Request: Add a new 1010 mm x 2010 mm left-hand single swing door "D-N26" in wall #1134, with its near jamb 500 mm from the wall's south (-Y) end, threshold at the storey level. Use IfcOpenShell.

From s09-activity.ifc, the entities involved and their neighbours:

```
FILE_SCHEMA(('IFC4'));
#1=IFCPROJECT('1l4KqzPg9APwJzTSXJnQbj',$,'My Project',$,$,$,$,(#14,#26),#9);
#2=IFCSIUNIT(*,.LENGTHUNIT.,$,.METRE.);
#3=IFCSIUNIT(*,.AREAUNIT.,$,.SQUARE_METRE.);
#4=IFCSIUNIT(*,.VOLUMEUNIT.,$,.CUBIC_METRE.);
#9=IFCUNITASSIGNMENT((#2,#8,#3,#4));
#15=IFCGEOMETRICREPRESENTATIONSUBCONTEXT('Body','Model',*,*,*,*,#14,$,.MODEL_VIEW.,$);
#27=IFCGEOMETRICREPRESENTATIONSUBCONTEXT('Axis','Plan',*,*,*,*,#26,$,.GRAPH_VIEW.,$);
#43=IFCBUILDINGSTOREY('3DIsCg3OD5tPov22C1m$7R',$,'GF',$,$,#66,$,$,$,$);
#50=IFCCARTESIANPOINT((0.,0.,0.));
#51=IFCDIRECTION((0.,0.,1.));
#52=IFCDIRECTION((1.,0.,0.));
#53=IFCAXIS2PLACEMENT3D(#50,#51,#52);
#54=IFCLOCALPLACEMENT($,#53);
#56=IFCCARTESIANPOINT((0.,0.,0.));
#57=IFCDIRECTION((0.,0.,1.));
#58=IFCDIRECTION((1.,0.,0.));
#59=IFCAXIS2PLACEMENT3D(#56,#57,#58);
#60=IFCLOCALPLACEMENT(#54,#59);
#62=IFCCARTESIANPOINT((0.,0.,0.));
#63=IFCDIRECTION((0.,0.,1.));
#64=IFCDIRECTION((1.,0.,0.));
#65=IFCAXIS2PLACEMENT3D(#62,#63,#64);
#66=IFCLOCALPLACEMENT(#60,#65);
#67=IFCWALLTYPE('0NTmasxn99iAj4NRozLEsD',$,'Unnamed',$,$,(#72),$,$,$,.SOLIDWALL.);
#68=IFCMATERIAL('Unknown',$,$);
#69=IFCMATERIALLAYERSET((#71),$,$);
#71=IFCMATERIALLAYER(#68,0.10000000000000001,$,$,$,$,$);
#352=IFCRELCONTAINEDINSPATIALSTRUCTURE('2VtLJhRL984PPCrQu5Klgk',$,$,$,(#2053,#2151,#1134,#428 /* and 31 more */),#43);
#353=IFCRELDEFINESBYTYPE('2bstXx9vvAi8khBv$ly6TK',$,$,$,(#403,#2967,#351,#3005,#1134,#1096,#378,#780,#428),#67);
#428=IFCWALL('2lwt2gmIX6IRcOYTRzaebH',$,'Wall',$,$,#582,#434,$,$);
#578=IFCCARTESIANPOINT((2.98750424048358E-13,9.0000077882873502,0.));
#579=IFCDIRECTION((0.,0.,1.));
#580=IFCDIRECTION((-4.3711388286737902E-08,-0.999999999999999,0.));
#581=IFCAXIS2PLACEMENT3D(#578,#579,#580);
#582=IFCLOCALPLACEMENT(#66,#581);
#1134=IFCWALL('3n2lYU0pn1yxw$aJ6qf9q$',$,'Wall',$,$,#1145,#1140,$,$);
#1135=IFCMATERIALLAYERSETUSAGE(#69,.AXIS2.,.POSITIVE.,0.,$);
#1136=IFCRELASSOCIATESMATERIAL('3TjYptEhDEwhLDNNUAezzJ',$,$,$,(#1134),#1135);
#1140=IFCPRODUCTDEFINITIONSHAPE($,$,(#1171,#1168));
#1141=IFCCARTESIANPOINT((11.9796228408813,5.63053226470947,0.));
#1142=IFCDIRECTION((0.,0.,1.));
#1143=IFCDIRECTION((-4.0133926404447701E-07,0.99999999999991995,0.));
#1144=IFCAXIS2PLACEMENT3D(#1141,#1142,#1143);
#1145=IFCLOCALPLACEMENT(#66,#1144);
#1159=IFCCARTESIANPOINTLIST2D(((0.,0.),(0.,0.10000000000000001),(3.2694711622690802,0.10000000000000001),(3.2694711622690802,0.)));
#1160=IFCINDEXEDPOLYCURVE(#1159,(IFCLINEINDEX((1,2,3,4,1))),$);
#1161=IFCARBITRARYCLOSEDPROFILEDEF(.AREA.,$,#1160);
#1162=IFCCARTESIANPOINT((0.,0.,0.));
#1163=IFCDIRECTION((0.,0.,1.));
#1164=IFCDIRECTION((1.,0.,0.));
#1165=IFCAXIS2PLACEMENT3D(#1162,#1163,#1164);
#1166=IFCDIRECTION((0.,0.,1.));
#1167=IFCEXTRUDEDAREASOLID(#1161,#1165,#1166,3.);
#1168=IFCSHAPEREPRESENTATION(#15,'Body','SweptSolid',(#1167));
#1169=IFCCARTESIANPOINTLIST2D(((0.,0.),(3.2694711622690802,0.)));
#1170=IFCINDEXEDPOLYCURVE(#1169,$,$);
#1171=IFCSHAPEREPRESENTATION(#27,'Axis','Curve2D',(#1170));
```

```python
import numpy as np
import ifcopenshell
import ifcopenshell.api.feature
import ifcopenshell.api.geometry
import ifcopenshell.api.root
import ifcopenshell.api.spatial
import ifcopenshell.geom
import ifcopenshell.util.element
import ifcopenshell.util.placement
import ifcopenshell.util.representation
import ifcopenshell.util.shape
import ifcopenshell.util.unit

model = ifcopenshell.open("s09-activity.ifc")
unit_scale = ifcopenshell.util.unit.calculate_unit_scale(model)
settings = ifcopenshell.geom.settings()


def volume(element):
    """Net volume in cubic metres, openings subtracted."""
    shape = ifcopenshell.geom.create_shape(settings, element)
    return ifcopenshell.util.shape.get_volume(shape.geometry)


wall = model.by_id(1134)
storey = ifcopenshell.util.element.get_container(wall, ifc_class="IfcBuildingStorey")
context = ifcopenshell.util.representation.get_context(model, "Model", "Body", "MODEL_VIEW")
before = volume(wall)

width, height, from_end, sill = 1.01, 2.01, 0.5, 0.0  # metres

# The wall runs along its own X axis, and the end named is its -X end.
wall_shape = ifcopenshell.geom.create_shape(settings, wall)
x, y, z = ifcopenshell.util.shape.get_vertices(wall_shape.geometry).T
start = x.min() + from_end
face, thickness = float(y.min()), float(y.max() - y.min())
wall_matrix = ifcopenshell.util.placement.get_local_placement(wall.ObjectPlacement)
level = ifcopenshell.util.placement.get_local_placement(storey.ObjectPlacement)[2, 3]


def in_wall(x, y):
    """Placement at x, y metres in the wall's axes, at sill height."""
    matrix = wall_matrix.copy()
    matrix[:, 3] = wall_matrix @ np.array([x / unit_scale, y / unit_scale, 0.0, 1.0])
    matrix[2, 3] = level + sill / unit_scale
    return matrix


# Opening: a box that overshoots both wall faces by 50 mm.
opening = ifcopenshell.api.root.create_entity(model, ifc_class="IfcOpeningElement", predefined_type="OPENING")
box = ifcopenshell.api.geometry.add_wall_representation(
    model, context=context, length=width, height=height, thickness=thickness + 0.1
)
ifcopenshell.api.geometry.assign_representation(model, product=opening, representation=box)
ifcopenshell.api.geometry.edit_object_placement(model, product=opening, matrix=in_wall(start, face - 0.05), is_si=False)
ifcopenshell.api.feature.add_feature(model, feature=opening, element=wall)

door = ifcopenshell.api.root.create_entity(model, ifc_class="IfcDoor", name="D-N26", predefined_type="DOOR")
door.OverallWidth, door.OverallHeight = width / unit_scale, height / unit_scale
door.OperationType = "SINGLE_SWING_LEFT"
body = ifcopenshell.api.geometry.add_door_representation(
    model,
    context=context,
    overall_width=door.OverallWidth,
    overall_height=door.OverallHeight,
    operation_type="SINGLE_SWING_LEFT",
    lining_properties={"LiningDepth": thickness / unit_scale, "ThresholdDepth": thickness / unit_scale},
)
ifcopenshell.api.geometry.assign_representation(model, product=door, representation=body)
ifcopenshell.api.spatial.assign_container(model, products=[door], relating_structure=storey)
ifcopenshell.api.feature.add_filling(model, opening=opening, element=door)

# The lining spans the wall, so the door starts at the wall face.
ifcopenshell.api.geometry.edit_object_placement(model, product=door, matrix=in_wall(start, face), is_si=False)

after = volume(wall)

print(f"wall volume {before:.3f} -> {after:.3f} m3")

model.write("s09-activity_v2.ifc")
```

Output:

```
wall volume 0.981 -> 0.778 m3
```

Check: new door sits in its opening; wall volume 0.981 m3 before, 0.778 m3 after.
